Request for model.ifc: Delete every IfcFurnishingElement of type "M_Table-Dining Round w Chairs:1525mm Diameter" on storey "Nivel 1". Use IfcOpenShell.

First a look at what the model holds.

```python
import ifcopenshell
import ifcopenshell.util.element

model = ifcopenshell.open("model.ifc")
print(model.schema)
storey = next(s for s in model.by_type("IfcBuildingStorey") if s.Name == "Nivel 1")
furniture = [e for e in ifcopenshell.util.element.get_decomposition(storey) if e.is_a("IfcFurnishingElement")]
seen = {}
for e in furniture:
    element_type = ifcopenshell.util.element.get_type(e)
    name = element_type.Name if element_type not in (None, e) else None
    seen[name] = seen.get(name, 0) + 1
for name, count in sorted(seen.items(), key=str):
    print(count, "x", name)
```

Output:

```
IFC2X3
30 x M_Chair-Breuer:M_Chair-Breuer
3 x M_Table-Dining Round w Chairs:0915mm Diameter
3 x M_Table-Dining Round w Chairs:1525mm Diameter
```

```python
import ifcopenshell
import ifcopenshell.api.root
import ifcopenshell.util.element

model = ifcopenshell.open("model.ifc")

storey = next(s for s in model.by_type("IfcBuildingStorey") if s.Name == "Nivel 1")
furniture = [e for e in ifcopenshell.util.element.get_decomposition(storey) if e.is_a("IfcFurnishingElement")]
targets = [e for e in furniture if (t := ifcopenshell.util.element.get_type(e)) not in (None, e) and t.Name == "M_Table-Dining Round w Chairs:1525mm Diameter"]

for e in targets:
    ifcopenshell.api.root.remove_product(model, product=e)
print(len(targets), "removed")

model.write("model_v2.ifc")
```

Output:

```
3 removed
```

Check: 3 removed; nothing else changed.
